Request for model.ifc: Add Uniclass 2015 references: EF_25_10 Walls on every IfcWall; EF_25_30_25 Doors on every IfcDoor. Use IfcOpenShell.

First a look at what the model holds.

```python
import ifcopenshell

model = ifcopenshell.open("model.ifc")
print(model.schema)
print("classifications:", [c.Name for c in model.by_type("IfcClassification")])
for ifc_class in ("IfcDoor", "IfcRoof", "IfcStair", "IfcWall", "IfcWindow"):
    print(ifc_class, len(model.by_type(ifc_class)))
```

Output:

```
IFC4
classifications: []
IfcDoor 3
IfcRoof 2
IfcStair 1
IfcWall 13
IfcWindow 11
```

```python
import ifcopenshell
import ifcopenshell.api.classification

model = ifcopenshell.open("model.ifc")

system = ifcopenshell.api.classification.add_classification(model, classification="Uniclass 2015")

codes = {
    "IfcWall": ("EF_25_10", "Walls"),
    "IfcDoor": ("EF_25_30_25", "Doors"),
}
for ifc_class, (code, name) in codes.items():
    products = model.by_type(ifc_class)
    ifcopenshell.api.classification.add_reference(
        model, products=products, classification=system, identification=code, name=name
    )
    print(code, len(products))

model.write("model-out.ifc")
```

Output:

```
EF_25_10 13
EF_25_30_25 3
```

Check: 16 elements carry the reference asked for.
